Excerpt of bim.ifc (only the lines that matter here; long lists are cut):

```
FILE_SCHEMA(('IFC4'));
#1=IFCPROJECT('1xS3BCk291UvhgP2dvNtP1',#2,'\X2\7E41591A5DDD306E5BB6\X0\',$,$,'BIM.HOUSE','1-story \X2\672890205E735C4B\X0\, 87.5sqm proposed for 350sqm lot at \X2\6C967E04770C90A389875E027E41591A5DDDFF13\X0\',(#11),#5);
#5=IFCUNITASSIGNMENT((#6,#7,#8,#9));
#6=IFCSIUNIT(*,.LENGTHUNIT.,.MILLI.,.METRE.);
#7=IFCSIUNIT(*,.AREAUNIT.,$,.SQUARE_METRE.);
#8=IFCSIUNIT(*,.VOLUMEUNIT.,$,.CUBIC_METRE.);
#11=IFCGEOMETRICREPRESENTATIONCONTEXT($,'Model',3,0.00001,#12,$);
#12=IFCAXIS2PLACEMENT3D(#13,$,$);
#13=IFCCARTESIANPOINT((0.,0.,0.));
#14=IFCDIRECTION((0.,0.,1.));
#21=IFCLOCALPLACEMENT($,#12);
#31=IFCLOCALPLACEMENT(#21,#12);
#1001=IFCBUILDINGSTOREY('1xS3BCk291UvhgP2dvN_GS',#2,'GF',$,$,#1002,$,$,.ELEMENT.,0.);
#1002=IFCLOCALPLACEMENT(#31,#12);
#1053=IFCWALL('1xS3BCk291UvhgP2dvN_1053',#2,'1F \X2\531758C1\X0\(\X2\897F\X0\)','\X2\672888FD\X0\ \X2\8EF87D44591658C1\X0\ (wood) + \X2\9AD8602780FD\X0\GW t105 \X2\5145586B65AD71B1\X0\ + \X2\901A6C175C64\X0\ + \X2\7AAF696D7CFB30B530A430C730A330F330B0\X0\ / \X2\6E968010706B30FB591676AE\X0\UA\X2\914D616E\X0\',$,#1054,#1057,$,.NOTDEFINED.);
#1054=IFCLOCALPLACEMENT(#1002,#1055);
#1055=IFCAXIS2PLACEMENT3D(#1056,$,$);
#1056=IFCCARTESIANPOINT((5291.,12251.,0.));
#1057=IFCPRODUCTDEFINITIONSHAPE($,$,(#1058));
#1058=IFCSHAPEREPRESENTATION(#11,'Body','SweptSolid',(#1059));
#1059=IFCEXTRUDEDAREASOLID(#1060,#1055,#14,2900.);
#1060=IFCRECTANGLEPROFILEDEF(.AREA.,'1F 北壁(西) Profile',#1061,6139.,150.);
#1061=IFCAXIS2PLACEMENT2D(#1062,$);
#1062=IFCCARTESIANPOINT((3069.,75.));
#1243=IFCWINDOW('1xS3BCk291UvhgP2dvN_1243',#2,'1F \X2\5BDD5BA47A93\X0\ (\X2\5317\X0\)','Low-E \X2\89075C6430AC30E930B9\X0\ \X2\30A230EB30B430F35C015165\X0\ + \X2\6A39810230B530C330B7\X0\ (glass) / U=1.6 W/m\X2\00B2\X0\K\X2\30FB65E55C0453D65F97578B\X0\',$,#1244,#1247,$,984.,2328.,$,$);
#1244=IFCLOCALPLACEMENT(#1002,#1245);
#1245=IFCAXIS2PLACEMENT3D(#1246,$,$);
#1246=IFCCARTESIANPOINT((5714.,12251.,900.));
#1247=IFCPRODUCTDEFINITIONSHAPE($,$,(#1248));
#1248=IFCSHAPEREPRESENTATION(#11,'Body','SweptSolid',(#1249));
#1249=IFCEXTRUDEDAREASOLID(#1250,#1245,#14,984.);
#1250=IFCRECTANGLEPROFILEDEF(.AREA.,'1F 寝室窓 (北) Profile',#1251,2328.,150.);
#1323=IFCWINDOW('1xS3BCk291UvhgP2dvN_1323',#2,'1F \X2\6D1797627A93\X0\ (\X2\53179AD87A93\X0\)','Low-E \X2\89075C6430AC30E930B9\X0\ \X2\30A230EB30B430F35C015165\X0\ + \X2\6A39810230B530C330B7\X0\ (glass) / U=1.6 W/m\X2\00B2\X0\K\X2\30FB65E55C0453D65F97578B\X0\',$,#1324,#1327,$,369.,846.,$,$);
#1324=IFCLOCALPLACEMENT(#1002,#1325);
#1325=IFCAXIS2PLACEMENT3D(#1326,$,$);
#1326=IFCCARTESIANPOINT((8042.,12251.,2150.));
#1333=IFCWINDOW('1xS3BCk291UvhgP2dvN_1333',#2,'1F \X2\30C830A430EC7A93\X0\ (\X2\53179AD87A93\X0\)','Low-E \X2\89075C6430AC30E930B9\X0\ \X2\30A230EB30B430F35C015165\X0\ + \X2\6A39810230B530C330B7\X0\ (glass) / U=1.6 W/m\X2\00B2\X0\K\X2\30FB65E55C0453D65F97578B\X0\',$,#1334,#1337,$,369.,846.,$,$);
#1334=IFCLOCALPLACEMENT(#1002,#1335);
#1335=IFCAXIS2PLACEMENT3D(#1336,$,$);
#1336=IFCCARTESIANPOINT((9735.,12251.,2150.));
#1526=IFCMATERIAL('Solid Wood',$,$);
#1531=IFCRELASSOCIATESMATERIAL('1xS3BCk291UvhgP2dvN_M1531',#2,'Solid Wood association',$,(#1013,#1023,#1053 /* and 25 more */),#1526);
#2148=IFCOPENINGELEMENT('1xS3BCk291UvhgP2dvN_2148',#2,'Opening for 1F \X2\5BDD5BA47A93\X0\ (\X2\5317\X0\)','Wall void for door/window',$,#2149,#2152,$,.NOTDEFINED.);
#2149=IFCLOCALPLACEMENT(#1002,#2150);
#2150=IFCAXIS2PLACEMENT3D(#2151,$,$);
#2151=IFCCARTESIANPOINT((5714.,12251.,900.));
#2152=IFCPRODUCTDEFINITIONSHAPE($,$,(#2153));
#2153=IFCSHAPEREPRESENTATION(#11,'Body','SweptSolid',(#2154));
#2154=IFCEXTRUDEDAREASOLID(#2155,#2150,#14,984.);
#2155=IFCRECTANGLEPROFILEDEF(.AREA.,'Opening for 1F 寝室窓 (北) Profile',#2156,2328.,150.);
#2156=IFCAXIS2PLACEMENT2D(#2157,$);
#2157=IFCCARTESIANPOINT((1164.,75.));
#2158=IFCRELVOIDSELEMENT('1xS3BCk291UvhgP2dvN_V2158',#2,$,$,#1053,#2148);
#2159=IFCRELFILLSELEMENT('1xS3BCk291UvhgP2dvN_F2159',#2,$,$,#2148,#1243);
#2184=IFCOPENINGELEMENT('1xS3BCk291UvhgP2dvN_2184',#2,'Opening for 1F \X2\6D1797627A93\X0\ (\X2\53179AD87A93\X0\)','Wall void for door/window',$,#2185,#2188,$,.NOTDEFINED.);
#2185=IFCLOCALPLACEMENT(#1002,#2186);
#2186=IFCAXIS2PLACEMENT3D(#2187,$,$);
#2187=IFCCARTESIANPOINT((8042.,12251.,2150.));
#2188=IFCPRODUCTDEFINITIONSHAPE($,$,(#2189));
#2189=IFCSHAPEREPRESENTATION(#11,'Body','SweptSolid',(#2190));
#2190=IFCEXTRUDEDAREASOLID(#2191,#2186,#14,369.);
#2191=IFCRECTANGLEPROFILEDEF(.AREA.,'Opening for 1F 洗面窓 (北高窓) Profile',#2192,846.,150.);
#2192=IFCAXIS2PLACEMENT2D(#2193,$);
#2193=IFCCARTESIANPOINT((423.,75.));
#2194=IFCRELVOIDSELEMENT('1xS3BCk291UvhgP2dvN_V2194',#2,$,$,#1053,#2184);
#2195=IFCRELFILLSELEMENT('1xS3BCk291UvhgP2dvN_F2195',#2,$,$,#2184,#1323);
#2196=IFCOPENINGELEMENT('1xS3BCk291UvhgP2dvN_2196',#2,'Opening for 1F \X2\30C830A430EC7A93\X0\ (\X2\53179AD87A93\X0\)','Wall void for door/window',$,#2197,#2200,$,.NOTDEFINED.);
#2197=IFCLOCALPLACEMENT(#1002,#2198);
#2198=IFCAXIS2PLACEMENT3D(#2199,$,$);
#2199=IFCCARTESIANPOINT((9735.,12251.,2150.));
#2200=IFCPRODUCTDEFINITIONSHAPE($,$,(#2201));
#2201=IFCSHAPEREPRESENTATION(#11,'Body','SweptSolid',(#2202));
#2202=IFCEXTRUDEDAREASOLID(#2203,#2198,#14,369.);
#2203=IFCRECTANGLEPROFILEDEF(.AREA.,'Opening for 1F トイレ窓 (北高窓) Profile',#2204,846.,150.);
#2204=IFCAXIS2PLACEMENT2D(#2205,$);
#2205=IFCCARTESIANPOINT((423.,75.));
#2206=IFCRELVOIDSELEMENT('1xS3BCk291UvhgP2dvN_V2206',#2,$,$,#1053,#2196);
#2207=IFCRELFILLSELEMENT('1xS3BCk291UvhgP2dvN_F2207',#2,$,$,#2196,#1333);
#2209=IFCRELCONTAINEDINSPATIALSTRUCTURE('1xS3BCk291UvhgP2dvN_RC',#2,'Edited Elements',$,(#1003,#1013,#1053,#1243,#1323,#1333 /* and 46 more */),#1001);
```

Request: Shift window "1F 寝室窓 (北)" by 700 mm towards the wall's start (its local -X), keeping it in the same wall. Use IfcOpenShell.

```python
import ifcopenshell
import ifcopenshell.api.geometry
import ifcopenshell.util.placement

model = ifcopenshell.open("bim.ifc")

window = model.by_guid("1xS3BCk291UvhgP2dvN_1243")
opening = window.FillsVoids[0].RelatingOpeningElement
wall = opening.VoidsElements[0].RelatingBuildingElement

wall_matrix = ifcopenshell.util.placement.get_local_placement(wall.ObjectPlacement)
shift = wall_matrix[:3, 0] * -700.0
before = ifcopenshell.util.placement.get_local_placement(window.ObjectPlacement)[:3, 3].copy()

# The window is not placed relative to its opening, so move both.
for product in (opening, window):
    matrix = ifcopenshell.util.placement.get_local_placement(product.ObjectPlacement)
    matrix[:3, 3] += shift
    ifcopenshell.api.geometry.edit_object_placement(model, product=product, matrix=matrix, is_si=False)

after = ifcopenshell.util.placement.get_local_placement(window.ObjectPlacement)[:3, 3]
print("window moved by", (after - before).round(3) + 0.0)

model.write("bim_rev.ifc")
```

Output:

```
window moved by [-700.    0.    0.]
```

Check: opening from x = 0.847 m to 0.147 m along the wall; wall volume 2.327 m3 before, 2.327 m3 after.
